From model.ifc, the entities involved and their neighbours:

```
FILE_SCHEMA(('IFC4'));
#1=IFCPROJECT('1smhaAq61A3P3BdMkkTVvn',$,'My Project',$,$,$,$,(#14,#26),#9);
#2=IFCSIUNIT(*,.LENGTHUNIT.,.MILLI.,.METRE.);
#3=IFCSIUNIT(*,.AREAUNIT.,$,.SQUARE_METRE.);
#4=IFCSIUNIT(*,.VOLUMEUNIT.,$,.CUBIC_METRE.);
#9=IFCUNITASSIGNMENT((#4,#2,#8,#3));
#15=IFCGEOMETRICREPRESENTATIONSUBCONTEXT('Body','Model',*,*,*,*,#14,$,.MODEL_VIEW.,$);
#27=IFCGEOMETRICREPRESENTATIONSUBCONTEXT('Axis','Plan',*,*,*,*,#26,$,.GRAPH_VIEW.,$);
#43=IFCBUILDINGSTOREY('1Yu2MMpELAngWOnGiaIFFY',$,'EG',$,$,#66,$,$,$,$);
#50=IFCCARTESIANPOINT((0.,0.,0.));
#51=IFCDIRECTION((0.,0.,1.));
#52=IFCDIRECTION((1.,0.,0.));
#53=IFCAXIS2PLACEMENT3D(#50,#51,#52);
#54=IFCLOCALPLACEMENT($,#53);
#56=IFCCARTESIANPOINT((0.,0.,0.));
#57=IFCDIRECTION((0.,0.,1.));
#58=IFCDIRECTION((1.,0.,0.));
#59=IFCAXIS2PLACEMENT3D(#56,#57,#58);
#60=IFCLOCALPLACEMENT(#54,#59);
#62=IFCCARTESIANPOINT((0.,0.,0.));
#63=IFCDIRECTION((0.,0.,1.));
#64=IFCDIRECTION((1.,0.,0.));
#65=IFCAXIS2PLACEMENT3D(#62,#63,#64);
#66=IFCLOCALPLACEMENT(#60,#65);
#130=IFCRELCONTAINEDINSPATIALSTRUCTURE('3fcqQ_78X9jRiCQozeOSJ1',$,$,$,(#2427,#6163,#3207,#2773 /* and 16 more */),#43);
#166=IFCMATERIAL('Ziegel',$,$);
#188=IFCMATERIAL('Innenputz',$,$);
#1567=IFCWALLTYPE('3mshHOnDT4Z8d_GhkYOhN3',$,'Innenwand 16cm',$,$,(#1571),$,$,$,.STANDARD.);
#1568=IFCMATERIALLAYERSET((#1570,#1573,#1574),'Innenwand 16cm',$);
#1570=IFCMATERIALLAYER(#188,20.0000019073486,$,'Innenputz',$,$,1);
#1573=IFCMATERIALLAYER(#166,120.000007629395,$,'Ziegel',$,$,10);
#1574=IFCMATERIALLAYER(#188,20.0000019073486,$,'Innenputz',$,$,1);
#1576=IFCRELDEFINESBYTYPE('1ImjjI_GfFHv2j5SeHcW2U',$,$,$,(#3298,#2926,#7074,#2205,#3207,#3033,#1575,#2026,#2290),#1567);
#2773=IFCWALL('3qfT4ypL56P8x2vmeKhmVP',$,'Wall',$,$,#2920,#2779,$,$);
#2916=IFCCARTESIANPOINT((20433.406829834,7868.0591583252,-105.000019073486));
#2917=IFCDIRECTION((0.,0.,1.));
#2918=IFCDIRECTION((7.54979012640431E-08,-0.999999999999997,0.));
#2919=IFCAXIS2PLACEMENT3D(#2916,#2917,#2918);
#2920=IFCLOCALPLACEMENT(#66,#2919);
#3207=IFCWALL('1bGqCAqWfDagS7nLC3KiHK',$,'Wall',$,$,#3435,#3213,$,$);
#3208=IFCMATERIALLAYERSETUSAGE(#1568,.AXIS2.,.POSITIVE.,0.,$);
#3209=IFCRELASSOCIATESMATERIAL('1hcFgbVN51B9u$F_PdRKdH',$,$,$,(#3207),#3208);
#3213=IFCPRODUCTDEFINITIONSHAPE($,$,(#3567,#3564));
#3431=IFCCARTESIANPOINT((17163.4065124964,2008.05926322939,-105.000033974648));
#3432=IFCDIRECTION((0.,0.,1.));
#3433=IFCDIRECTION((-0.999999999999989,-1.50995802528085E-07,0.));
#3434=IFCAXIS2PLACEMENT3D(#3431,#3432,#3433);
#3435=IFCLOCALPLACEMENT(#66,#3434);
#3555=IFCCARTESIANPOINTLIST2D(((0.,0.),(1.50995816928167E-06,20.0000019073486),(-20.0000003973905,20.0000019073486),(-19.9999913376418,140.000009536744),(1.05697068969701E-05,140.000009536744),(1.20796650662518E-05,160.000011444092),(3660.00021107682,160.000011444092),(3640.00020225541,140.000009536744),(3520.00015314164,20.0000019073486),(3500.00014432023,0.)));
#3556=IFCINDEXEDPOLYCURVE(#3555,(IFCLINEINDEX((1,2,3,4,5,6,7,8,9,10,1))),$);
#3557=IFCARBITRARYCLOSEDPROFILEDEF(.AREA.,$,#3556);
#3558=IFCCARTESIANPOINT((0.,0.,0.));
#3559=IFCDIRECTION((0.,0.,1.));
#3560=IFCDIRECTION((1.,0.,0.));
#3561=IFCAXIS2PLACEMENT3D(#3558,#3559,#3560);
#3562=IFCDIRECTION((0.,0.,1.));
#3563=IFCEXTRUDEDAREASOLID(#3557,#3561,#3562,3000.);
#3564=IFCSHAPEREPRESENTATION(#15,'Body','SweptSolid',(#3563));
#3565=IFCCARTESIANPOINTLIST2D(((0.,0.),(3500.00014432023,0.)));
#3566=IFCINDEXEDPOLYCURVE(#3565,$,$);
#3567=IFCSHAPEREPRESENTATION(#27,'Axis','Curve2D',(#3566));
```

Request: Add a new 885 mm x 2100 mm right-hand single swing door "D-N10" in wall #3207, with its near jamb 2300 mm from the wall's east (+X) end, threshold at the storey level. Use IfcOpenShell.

```python
import numpy as np
import ifcopenshell
import ifcopenshell.api.feature
import ifcopenshell.api.geometry
import ifcopenshell.api.root
import ifcopenshell.api.spatial
import ifcopenshell.geom
import ifcopenshell.util.element
import ifcopenshell.util.placement
import ifcopenshell.util.representation
import ifcopenshell.util.shape
import ifcopenshell.util.unit

model = ifcopenshell.open("model.ifc")
unit_scale = ifcopenshell.util.unit.calculate_unit_scale(model)
settings = ifcopenshell.geom.settings()


def volume(element):
    """Net volume in cubic metres, openings subtracted."""
    shape = ifcopenshell.geom.create_shape(settings, element)
    return ifcopenshell.util.shape.get_volume(shape.geometry)


wall = model.by_guid("1bGqCAqWfDagS7nLC3KiHK")
storey = ifcopenshell.util.element.get_container(wall, ifc_class="IfcBuildingStorey")
context = ifcopenshell.util.representation.get_context(model, "Model", "Body", "MODEL_VIEW")
before = volume(wall)

width, height, from_end, sill = 0.885, 2.1, 2.3, 0.0  # metres

# The wall runs along its own X axis, and the end named is its -X end.
wall_shape = ifcopenshell.geom.create_shape(settings, wall)
x, y, z = ifcopenshell.util.shape.get_vertices(wall_shape.geometry).T
start = x.min() + from_end
face, thickness = float(y.min()), float(y.max() - y.min())
wall_matrix = ifcopenshell.util.placement.get_local_placement(wall.ObjectPlacement)
level = ifcopenshell.util.placement.get_local_placement(storey.ObjectPlacement)[2, 3]


def in_wall(x, y):
    """Placement at x, y metres in the wall's axes, at sill height."""
    matrix = wall_matrix.copy()
    matrix[:, 3] = wall_matrix @ np.array([x / unit_scale, y / unit_scale, 0.0, 1.0])
    matrix[2, 3] = level + sill / unit_scale
    return matrix


# Opening: a box that overshoots both wall faces by 50 mm.
opening = ifcopenshell.api.root.create_entity(model, ifc_class="IfcOpeningElement", predefined_type="OPENING")
box = ifcopenshell.api.geometry.add_wall_representation(
    model, context=context, length=width, height=height, thickness=thickness + 0.1
)
ifcopenshell.api.geometry.assign_representation(model, product=opening, representation=box)
ifcopenshell.api.geometry.edit_object_placement(model, product=opening, matrix=in_wall(start, face - 0.05), is_si=False)
ifcopenshell.api.feature.add_feature(model, feature=opening, element=wall)

door = ifcopenshell.api.root.create_entity(model, ifc_class="IfcDoor", name="D-N10", predefined_type="DOOR")
door.OverallWidth, door.OverallHeight = width / unit_scale, height / unit_scale
door.OperationType = "SINGLE_SWING_RIGHT"
body = ifcopenshell.api.geometry.add_door_representation(
    model,
    context=context,
    overall_width=door.OverallWidth,
    overall_height=door.OverallHeight,
    operation_type="SINGLE_SWING_RIGHT",
    lining_properties={"LiningDepth": thickness / unit_scale, "ThresholdDepth": thickness / unit_scale},
)
ifcopenshell.api.geometry.assign_representation(model, product=door, representation=body)
ifcopenshell.api.spatial.assign_container(model, products=[door], relating_structure=storey)
ifcopenshell.api.feature.add_filling(model, opening=opening, element=door)

# The lining spans the wall, so the door starts at the wall face.
ifcopenshell.api.geometry.edit_object_placement(model, product=door, matrix=in_wall(start, face), is_si=False)

after = volume(wall)

print(f"wall volume {before:.3f} -> {after:.3f} m3")

model.write("model_updated.ifc")
```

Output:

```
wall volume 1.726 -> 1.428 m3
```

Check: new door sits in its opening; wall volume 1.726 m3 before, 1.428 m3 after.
